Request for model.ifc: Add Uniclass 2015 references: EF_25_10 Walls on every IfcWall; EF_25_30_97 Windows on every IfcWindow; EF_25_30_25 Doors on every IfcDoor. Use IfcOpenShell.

First a look at what the model holds.

```python
import ifcopenshell

model = ifcopenshell.open("model.ifc")
print(model.schema)
print("classifications:", [c.Name for c in model.by_type("IfcClassification")])
for ifc_class in ("IfcDoor", "IfcRoof", "IfcStair", "IfcWall", "IfcWindow"):
    print(ifc_class, len(model.by_type(ifc_class)))
```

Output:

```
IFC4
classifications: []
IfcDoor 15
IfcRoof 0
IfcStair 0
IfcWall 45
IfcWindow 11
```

```python
import ifcopenshell
import ifcopenshell.api.classification

model = ifcopenshell.open("model.ifc")

system = ifcopenshell.api.classification.add_classification(model, classification="Uniclass 2015")

codes = {
    "IfcWall": ("EF_25_10", "Walls"),
    "IfcWindow": ("EF_25_30_97", "Windows"),
    "IfcDoor": ("EF_25_30_25", "Doors"),
}
for ifc_class, (code, name) in codes.items():
    products = model.by_type(ifc_class)
    ifcopenshell.api.classification.add_reference(
        model, products=products, classification=system, identification=code, name=name
    )
    print(code, len(products))

model.write("model_v2.ifc")
```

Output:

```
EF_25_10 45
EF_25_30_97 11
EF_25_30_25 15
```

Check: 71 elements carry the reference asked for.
